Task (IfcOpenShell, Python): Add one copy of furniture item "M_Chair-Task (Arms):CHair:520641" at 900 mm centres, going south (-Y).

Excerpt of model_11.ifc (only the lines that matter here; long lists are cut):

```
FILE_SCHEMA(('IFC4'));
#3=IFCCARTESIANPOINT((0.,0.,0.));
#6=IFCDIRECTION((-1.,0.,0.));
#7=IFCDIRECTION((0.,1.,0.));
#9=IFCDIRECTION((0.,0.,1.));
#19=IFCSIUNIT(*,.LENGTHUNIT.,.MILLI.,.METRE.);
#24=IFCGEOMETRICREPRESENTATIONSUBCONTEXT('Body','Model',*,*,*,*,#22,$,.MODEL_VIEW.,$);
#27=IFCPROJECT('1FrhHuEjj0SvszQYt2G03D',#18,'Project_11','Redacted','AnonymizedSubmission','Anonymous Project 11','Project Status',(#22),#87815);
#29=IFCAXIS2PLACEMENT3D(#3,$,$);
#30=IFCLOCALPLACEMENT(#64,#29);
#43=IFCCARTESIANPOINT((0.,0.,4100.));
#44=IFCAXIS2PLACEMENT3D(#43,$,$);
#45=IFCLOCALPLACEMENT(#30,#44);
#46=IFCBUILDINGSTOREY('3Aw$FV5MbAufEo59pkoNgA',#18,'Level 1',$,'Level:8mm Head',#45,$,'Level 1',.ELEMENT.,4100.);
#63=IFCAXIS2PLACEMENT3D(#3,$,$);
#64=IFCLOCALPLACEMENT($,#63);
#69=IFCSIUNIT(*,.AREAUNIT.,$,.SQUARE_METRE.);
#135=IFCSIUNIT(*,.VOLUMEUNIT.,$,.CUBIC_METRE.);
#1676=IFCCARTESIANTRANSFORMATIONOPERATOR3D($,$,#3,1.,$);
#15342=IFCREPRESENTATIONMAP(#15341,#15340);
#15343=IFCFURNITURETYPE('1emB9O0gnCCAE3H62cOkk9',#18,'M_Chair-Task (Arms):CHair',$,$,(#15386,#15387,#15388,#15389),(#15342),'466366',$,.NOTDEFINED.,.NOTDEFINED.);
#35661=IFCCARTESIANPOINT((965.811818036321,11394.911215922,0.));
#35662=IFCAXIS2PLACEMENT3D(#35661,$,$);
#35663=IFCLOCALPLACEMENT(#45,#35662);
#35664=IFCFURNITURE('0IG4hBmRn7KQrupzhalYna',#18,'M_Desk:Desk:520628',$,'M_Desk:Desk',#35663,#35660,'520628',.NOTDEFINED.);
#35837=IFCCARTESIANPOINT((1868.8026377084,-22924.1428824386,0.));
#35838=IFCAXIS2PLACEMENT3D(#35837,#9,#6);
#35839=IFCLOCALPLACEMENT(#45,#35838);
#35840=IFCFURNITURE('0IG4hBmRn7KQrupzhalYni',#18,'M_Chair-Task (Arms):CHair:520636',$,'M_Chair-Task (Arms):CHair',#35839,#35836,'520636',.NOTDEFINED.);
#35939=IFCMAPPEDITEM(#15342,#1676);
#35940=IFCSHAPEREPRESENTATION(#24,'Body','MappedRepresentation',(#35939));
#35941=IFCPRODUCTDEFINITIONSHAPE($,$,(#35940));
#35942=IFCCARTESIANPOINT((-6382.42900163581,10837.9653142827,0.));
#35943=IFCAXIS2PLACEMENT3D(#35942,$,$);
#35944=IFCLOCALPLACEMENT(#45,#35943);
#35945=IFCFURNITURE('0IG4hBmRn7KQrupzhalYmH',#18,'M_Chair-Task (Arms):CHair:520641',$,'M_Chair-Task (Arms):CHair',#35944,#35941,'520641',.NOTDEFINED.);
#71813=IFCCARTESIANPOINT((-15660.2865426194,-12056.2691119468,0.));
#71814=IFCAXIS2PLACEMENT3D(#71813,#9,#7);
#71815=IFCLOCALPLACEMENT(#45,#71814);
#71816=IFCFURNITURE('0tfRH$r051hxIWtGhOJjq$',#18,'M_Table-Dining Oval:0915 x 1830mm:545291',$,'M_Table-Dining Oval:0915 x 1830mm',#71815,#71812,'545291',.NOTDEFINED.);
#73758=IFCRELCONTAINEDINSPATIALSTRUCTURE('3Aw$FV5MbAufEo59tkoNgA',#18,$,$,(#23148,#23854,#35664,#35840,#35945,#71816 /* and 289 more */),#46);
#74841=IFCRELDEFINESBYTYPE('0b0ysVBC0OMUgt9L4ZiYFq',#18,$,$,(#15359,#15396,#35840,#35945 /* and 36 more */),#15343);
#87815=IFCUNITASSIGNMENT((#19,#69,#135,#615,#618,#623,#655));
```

```python
import numpy as np
import ifcopenshell
import ifcopenshell.api.geometry
import ifcopenshell.api.root
import ifcopenshell.util.element
import ifcopenshell.util.placement

model = ifcopenshell.open("model_11.ifc")


def reuse_history(source, copy):
    """copy_class also copies each property set's owner history, people and application; keep the originals."""
    for rel in copy.IsDefinedBy:
        if rel.is_a("IfcRelDefinesByProperties") and (history := rel.RelatingPropertyDefinition.OwnerHistory):
            rel.RelatingPropertyDefinition.OwnerHistory = source.OwnerHistory
            ifcopenshell.util.element.remove_deep2(model, history)


source = model.by_guid("0IG4hBmRn7KQrupzhalYmH")
base = ifcopenshell.util.placement.get_local_placement(source.ObjectPlacement)
step = np.array([0.0, -1.0, 0.0]) * 900.0

for i in range(1, 2):
    copy = ifcopenshell.api.root.copy_class(model, product=source)
    copy.Representation = ifcopenshell.util.element.copy_deep(
        model, source.Representation, exclude=["IfcGeometricRepresentationContext", "IfcRepresentationMap"]
    )
    copy.Name = "M_Chair-Task (Arms):CHair"
    copy.Tag = None
    reuse_history(source, copy)
    matrix = base.copy()
    matrix[:3, 3] += i * step
    print("added at", matrix[:3, 3].round(3) + 0.0)
    ifcopenshell.api.geometry.edit_object_placement(model, product=copy, matrix=matrix, is_si=False)

model.write("model_11-out.ifc")
```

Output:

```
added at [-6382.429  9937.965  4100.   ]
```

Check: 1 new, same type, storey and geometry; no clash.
